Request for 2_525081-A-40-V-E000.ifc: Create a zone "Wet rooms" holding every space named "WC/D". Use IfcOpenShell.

First a look at what the model holds.

```python
import ifcopenshell

model = ifcopenshell.open("2_525081-A-40-V-E000.ifc")
print(model.schema)
seen = {}
for space in model.by_type("IfcSpace"):
    seen[space.LongName] = seen.get(space.LongName, 0) + 1
for name, count in sorted(seen.items(), key=str):
    print(count, "x", name)
print("zones:", [z.Name for z in model.by_type("IfcZone")][:20])
```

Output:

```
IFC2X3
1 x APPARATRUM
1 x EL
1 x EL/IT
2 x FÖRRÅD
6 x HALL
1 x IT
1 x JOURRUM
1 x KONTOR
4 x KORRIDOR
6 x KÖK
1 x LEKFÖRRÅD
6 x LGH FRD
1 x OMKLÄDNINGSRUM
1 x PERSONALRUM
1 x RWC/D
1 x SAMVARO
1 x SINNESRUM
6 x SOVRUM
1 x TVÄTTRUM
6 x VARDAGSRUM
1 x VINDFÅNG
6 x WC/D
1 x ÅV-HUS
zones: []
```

```python
import ifcopenshell
import ifcopenshell.api.group
import ifcopenshell.api.root

model = ifcopenshell.open("2_525081-A-40-V-E000.ifc")

names = {"WC/D"}
spaces = [s for s in model.by_type("IfcSpace") if s.LongName in names]

zone = ifcopenshell.api.root.create_entity(model, ifc_class="IfcZone", name="Wet rooms")
ifcopenshell.api.group.assign_group(model, products=spaces, group=zone)
print(len(spaces), "spaces in", zone.Name)

model.write("2_525081-A-40-V-E000_updated.ifc")
```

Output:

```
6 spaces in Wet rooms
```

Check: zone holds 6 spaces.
